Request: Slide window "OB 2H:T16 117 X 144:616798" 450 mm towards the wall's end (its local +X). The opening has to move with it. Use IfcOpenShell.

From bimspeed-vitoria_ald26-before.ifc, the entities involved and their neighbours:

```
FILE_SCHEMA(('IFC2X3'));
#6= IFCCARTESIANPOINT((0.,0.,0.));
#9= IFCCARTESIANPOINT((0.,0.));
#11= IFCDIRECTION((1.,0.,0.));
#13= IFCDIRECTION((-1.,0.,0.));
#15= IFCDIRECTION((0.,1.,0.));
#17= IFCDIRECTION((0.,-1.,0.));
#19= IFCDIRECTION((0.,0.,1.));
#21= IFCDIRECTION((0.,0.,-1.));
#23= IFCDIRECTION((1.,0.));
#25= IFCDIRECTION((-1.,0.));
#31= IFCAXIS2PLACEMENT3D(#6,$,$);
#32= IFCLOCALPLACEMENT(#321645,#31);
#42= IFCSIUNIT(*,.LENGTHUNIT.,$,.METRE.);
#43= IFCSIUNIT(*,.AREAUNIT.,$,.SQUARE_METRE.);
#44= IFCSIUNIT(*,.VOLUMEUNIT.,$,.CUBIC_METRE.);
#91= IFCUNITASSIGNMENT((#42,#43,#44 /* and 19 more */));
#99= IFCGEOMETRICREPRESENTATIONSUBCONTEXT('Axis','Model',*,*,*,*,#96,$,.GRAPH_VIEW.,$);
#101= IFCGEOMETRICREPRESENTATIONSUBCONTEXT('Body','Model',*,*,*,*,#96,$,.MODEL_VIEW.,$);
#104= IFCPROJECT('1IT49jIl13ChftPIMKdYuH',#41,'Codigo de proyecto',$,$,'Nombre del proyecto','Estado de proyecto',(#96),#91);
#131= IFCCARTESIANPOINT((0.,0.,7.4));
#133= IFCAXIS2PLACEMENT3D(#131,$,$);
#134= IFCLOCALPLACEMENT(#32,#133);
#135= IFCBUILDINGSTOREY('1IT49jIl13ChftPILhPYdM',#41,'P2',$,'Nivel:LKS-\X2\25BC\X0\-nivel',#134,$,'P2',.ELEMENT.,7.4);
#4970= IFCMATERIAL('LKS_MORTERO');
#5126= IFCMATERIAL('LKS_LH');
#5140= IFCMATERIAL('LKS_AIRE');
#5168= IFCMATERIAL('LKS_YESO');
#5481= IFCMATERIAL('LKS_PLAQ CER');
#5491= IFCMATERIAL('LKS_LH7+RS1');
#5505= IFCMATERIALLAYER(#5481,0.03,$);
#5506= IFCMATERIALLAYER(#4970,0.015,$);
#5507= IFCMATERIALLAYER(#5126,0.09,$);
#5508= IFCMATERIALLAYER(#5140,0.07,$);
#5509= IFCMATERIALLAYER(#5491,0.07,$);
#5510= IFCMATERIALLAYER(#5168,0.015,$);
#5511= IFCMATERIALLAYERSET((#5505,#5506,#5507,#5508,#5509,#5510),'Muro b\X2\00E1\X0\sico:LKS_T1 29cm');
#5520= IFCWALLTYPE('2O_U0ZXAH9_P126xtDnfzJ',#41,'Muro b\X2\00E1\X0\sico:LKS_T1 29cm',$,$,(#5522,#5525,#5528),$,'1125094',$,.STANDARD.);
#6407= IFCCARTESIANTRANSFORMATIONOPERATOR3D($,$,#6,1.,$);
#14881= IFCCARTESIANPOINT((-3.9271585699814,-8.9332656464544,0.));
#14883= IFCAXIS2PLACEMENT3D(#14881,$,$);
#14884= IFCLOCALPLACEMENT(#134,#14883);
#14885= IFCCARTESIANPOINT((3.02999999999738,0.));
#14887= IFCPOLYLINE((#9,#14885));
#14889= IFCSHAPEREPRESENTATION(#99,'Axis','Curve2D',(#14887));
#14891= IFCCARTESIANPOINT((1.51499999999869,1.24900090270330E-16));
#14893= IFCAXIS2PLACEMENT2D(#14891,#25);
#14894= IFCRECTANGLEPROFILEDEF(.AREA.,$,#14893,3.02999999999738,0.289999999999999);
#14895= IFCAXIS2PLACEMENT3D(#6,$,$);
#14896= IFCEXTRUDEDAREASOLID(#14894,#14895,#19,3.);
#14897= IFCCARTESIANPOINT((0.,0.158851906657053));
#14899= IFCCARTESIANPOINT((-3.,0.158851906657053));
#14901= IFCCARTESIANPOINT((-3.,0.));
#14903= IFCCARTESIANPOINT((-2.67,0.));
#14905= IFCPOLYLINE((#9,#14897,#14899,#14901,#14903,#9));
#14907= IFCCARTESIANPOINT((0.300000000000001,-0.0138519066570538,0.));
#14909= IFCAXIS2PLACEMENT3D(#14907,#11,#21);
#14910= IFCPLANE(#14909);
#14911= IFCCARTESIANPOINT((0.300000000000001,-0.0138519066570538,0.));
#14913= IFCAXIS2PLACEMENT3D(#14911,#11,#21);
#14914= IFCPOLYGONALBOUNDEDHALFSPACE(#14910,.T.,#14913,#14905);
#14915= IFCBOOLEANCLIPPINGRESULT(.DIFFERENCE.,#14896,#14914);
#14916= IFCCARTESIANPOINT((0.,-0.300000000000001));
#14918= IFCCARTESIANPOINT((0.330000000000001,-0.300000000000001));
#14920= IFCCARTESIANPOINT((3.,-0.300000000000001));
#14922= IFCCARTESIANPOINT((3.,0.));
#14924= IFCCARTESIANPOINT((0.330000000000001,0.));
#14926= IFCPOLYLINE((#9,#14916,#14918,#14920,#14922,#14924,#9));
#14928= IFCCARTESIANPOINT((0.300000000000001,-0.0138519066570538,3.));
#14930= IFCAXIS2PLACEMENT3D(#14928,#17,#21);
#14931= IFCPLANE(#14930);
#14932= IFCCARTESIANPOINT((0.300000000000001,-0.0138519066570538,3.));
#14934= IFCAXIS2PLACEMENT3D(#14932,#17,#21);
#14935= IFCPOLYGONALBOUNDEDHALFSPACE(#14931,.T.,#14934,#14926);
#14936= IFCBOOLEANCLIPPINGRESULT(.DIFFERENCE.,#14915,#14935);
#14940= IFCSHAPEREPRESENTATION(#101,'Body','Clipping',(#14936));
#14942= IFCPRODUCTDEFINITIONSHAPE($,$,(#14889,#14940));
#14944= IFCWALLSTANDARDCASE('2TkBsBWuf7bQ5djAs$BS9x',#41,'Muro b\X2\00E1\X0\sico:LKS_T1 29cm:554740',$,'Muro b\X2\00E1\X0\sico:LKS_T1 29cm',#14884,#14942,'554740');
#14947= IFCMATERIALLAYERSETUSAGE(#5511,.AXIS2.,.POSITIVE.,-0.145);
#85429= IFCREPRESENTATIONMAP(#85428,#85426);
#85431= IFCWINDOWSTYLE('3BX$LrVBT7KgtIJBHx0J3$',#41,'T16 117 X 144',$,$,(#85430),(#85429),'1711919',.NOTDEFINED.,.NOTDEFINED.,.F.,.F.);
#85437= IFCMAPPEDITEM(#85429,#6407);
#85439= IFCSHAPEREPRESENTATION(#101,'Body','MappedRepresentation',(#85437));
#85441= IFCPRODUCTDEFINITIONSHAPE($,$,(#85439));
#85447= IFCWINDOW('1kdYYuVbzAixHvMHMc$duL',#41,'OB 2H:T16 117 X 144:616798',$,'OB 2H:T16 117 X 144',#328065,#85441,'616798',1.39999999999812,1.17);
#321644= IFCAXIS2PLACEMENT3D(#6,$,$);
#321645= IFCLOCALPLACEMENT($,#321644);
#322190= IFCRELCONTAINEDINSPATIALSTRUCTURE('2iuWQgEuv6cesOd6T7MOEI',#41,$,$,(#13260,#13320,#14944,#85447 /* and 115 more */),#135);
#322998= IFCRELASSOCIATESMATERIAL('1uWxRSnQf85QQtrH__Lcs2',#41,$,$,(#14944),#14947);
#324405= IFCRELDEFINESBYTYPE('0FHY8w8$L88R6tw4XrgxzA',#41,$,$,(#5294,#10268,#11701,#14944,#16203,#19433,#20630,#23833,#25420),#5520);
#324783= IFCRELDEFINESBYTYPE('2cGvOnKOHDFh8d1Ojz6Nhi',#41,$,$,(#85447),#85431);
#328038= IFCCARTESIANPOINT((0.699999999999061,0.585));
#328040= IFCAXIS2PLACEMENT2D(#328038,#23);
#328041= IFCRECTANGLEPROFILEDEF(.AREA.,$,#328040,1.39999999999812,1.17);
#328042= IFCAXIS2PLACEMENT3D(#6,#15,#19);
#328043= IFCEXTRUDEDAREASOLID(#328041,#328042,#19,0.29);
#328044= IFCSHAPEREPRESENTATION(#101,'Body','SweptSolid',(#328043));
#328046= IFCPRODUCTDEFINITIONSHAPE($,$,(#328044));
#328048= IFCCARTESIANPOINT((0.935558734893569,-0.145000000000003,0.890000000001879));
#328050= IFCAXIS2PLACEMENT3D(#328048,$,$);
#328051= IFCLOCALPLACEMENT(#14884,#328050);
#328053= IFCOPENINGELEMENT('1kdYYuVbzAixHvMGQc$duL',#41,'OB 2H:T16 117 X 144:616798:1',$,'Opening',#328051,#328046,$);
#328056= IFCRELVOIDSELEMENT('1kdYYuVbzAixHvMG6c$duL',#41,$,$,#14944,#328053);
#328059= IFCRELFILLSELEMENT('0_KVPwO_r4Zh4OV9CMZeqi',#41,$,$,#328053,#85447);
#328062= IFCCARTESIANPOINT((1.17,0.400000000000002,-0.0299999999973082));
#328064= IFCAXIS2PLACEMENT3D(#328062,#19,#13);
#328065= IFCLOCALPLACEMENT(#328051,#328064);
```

```python
import ifcopenshell
import ifcopenshell.api.geometry
import ifcopenshell.util.placement
import ifcopenshell.util.unit

model = ifcopenshell.open("bimspeed-vitoria_ald26-before.ifc")
unit_scale = ifcopenshell.util.unit.calculate_unit_scale(model)

window = model.by_guid("1kdYYuVbzAixHvMHMc$duL")
opening = window.FillsVoids[0].RelatingOpeningElement
wall = opening.VoidsElements[0].RelatingBuildingElement

wall_matrix = ifcopenshell.util.placement.get_local_placement(wall.ObjectPlacement)
shift = wall_matrix[:3, 0] * 0.45 / unit_scale
before = ifcopenshell.util.placement.get_local_placement(window.ObjectPlacement)[:3, 3].copy()

# The window is placed relative to its opening, so it follows when the opening moves.
matrix = ifcopenshell.util.placement.get_local_placement(opening.ObjectPlacement)
matrix[:3, 3] += shift
ifcopenshell.api.geometry.edit_object_placement(
    model, product=opening, matrix=matrix, is_si=False, should_transform_children=True
)

after = ifcopenshell.util.placement.get_local_placement(window.ObjectPlacement)[:3, 3]
print("window moved by", (after - before).round(3) + 0.0)

model.write("bimspeed-vitoria_ald26-before_updated.ifc")
```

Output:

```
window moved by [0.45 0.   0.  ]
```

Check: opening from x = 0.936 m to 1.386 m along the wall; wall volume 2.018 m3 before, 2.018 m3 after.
